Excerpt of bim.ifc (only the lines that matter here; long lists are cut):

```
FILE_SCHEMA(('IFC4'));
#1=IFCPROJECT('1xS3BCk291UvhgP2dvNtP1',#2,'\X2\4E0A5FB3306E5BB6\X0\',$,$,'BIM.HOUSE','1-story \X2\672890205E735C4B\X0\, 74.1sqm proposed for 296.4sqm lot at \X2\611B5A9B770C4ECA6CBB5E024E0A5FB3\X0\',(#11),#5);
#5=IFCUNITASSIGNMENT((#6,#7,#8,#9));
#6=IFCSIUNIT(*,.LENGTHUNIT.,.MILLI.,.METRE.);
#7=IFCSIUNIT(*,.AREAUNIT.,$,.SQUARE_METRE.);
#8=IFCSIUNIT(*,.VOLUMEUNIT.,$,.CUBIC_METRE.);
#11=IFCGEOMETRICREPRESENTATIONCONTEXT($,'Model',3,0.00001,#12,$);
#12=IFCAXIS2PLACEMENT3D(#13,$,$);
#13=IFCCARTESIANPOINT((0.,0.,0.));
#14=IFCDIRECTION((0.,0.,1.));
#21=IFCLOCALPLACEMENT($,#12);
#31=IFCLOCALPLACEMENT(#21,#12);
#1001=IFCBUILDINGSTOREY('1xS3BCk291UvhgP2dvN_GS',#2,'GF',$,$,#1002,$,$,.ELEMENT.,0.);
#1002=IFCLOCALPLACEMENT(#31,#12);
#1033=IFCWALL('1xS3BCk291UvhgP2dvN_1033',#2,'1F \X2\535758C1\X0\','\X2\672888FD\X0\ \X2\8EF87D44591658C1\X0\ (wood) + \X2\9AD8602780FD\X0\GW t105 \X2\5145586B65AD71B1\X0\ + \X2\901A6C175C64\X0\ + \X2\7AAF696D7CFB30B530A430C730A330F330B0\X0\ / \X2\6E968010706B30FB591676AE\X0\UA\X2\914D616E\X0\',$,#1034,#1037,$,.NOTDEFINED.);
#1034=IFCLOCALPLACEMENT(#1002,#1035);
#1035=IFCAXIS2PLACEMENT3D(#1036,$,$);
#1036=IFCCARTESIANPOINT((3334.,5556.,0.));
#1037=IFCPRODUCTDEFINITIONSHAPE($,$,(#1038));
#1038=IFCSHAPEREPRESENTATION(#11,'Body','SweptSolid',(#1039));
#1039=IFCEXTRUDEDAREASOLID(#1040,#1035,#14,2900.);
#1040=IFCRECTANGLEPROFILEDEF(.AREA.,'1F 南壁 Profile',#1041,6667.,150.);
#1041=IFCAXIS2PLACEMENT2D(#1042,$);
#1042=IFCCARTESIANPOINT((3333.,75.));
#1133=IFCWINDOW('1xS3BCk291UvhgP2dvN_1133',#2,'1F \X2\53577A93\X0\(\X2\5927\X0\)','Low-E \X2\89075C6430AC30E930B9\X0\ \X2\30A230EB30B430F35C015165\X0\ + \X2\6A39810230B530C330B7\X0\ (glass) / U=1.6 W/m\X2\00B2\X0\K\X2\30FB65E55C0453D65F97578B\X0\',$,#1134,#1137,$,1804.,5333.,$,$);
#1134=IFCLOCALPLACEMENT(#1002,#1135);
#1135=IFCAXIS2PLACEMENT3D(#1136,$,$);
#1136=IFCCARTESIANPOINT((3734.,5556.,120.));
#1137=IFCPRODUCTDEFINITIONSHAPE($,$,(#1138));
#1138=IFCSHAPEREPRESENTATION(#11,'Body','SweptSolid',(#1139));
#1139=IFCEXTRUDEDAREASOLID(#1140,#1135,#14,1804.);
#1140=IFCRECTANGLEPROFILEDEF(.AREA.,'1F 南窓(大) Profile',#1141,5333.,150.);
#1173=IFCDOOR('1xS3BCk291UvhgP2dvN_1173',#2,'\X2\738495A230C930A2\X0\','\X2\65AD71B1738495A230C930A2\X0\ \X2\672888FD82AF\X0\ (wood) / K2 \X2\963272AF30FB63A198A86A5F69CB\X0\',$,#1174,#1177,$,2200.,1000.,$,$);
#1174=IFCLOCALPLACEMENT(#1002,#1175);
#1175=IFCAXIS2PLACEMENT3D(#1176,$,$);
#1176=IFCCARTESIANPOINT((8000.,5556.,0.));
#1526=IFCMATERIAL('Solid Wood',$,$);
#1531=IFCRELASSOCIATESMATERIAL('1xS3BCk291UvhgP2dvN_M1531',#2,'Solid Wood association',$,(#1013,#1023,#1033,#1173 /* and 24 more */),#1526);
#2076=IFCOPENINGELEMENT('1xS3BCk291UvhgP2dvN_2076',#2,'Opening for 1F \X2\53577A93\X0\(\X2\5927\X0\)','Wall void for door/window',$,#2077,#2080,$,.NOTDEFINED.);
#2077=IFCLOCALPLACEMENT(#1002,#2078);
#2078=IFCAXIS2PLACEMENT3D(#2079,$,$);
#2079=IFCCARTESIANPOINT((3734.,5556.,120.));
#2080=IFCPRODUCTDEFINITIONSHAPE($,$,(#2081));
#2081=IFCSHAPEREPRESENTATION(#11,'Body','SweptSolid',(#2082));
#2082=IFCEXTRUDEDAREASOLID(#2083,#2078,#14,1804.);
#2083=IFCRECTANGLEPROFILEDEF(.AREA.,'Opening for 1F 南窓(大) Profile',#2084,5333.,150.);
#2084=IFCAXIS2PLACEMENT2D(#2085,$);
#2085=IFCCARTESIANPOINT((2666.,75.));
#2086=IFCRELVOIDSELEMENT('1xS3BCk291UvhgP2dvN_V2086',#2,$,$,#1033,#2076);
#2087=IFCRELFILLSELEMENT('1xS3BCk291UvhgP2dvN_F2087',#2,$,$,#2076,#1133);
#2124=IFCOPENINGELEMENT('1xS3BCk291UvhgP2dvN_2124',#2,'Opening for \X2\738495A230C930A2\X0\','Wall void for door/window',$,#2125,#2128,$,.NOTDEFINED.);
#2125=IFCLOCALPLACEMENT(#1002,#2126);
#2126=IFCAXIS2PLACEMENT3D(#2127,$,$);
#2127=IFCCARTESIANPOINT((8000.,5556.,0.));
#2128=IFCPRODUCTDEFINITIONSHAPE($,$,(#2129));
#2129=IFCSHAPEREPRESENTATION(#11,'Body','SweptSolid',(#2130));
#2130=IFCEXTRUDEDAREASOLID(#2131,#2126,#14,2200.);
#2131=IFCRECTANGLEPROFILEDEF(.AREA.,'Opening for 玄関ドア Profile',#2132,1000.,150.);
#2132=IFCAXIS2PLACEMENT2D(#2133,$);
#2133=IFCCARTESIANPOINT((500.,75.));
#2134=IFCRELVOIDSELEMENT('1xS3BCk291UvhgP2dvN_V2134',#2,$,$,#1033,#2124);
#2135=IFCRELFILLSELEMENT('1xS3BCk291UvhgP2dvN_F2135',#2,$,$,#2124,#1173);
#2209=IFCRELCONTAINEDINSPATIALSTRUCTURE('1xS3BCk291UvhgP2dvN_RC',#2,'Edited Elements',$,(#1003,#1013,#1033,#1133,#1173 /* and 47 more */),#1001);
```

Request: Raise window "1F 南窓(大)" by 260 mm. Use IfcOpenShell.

```python
import numpy as np
import ifcopenshell
import ifcopenshell.api.geometry
import ifcopenshell.util.placement
import ifcopenshell.util.unit

model = ifcopenshell.open("bim.ifc")
unit_scale = ifcopenshell.util.unit.calculate_unit_scale(model)

window = model.by_guid("1xS3BCk291UvhgP2dvN_1133")
opening = window.FillsVoids[0].RelatingOpeningElement
dz = 0.26 / unit_scale

shift = np.array([0.0, 0.0, dz])
# The window is not placed relative to its opening, so move both.
for product in (opening, window):
    matrix = ifcopenshell.util.placement.get_local_placement(product.ObjectPlacement)
    matrix[:3, 3] += shift
    ifcopenshell.api.geometry.edit_object_placement(model, product=product, matrix=matrix, is_si=False)

print(f"moved by {dz * unit_scale:+.3f} m")

model.write("bim-out.ifc")
```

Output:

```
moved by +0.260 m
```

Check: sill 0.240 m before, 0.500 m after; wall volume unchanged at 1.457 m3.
